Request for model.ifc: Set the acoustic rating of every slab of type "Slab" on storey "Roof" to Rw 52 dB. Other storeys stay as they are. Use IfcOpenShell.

First a look at what the model holds.

```python
import ifcopenshell
import ifcopenshell.util.element

model = ifcopenshell.open("model.ifc")
print(model.schema)
storey = next(s for s in model.by_type("IfcBuildingStorey") if s.Name == "Roof")
slabs = [e for e in ifcopenshell.util.element.get_decomposition(storey) if e.is_a("IfcSlab")]
seen = {}
for e in slabs:
    element_type = ifcopenshell.util.element.get_type(e)
    key = (element_type.Name if element_type != e and element_type else None, ifcopenshell.util.element.get_pset(e, "Pset_SlabCommon", "AcousticRating"))
    seen[key] = seen.get(key, 0) + 1
for (name, value), count in sorted(seen.items(), key=str):
    print(count, "x", name, "|", value)
```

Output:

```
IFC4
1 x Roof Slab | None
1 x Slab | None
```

```python
import ifcopenshell
import ifcopenshell.api.pset
import ifcopenshell.util.element

model = ifcopenshell.open("model.ifc")

storey = next(s for s in model.by_type("IfcBuildingStorey") if s.Name == "Roof")
slabs = [e for e in ifcopenshell.util.element.get_decomposition(storey) if e.is_a("IfcSlab")]

count = 0
for e in slabs:
    element_type = ifcopenshell.util.element.get_type(e)
    if element_type in (None, e) or element_type.Name != "Slab":
        continue
    # add_pset returns the element's existing set when there is one.
    pset = ifcopenshell.api.pset.add_pset(model, product=e, name="Pset_SlabCommon")
    ifcopenshell.api.pset.edit_pset(model, pset=pset, properties={"AcousticRating": "Rw 52 dB"})
    count += 1

print(count, "slabs updated")

model.write("model_v2.ifc")
```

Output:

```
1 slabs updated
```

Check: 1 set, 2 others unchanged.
